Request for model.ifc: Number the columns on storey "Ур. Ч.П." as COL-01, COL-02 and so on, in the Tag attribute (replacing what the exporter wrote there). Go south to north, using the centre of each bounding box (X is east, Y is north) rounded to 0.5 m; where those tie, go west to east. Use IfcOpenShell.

First a look at what the model holds.

```python
import ifcopenshell
import ifcopenshell.util.element
import ifcopenshell.util.placement

model = ifcopenshell.open("model.ifc")
print(model.schema)
storey = next(s for s in model.by_type("IfcBuildingStorey") if s.Name == "Ур. Ч.П.")
columns = [e for e in ifcopenshell.util.element.get_decomposition(storey) if e.is_a("IfcColumn")]
for e in sorted(columns, key=lambda e: e.id()):
    origin = ifcopenshell.util.placement.get_local_placement(e.ObjectPlacement)[:3, 3]
    print(e.id(), e.Tag, e.Name, origin.round(2) + 0.0, sep=" | ")
```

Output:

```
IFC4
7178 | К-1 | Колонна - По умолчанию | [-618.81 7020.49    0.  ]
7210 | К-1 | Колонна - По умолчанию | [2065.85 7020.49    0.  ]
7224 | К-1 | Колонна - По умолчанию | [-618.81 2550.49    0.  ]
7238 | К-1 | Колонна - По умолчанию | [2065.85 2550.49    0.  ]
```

```python
import ifcopenshell
import ifcopenshell.geom
import ifcopenshell.util.element
import ifcopenshell.util.shape

model = ifcopenshell.open("model.ifc")
settings = ifcopenshell.geom.settings()
settings.set("use-world-coords", True)


def centre(element):
    shape = ifcopenshell.geom.create_shape(settings, element)
    return ifcopenshell.util.shape.get_bbox_centroid(shape.geometry)


storey = next(s for s in model.by_type("IfcBuildingStorey") if s.Name == "Ур. Ч.П.")
columns = [e for e in ifcopenshell.util.element.get_decomposition(storey) if e.is_a("IfcColumn")]

# Insertion points can sit at a corner or the storey origin, so sort by the geometry (in metres).
centres = {e: centre(e) for e in columns}
columns.sort(key=lambda e: (round(centres[e][1] / 0.5), centres[e][0]))

for i, e in enumerate(columns, start=1):
    number = f"COL-{i:02d}"
    e.Tag = number
    print(e.id(), number)

model.write("model-out.ifc")
```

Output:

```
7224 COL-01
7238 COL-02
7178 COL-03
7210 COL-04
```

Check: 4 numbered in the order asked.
